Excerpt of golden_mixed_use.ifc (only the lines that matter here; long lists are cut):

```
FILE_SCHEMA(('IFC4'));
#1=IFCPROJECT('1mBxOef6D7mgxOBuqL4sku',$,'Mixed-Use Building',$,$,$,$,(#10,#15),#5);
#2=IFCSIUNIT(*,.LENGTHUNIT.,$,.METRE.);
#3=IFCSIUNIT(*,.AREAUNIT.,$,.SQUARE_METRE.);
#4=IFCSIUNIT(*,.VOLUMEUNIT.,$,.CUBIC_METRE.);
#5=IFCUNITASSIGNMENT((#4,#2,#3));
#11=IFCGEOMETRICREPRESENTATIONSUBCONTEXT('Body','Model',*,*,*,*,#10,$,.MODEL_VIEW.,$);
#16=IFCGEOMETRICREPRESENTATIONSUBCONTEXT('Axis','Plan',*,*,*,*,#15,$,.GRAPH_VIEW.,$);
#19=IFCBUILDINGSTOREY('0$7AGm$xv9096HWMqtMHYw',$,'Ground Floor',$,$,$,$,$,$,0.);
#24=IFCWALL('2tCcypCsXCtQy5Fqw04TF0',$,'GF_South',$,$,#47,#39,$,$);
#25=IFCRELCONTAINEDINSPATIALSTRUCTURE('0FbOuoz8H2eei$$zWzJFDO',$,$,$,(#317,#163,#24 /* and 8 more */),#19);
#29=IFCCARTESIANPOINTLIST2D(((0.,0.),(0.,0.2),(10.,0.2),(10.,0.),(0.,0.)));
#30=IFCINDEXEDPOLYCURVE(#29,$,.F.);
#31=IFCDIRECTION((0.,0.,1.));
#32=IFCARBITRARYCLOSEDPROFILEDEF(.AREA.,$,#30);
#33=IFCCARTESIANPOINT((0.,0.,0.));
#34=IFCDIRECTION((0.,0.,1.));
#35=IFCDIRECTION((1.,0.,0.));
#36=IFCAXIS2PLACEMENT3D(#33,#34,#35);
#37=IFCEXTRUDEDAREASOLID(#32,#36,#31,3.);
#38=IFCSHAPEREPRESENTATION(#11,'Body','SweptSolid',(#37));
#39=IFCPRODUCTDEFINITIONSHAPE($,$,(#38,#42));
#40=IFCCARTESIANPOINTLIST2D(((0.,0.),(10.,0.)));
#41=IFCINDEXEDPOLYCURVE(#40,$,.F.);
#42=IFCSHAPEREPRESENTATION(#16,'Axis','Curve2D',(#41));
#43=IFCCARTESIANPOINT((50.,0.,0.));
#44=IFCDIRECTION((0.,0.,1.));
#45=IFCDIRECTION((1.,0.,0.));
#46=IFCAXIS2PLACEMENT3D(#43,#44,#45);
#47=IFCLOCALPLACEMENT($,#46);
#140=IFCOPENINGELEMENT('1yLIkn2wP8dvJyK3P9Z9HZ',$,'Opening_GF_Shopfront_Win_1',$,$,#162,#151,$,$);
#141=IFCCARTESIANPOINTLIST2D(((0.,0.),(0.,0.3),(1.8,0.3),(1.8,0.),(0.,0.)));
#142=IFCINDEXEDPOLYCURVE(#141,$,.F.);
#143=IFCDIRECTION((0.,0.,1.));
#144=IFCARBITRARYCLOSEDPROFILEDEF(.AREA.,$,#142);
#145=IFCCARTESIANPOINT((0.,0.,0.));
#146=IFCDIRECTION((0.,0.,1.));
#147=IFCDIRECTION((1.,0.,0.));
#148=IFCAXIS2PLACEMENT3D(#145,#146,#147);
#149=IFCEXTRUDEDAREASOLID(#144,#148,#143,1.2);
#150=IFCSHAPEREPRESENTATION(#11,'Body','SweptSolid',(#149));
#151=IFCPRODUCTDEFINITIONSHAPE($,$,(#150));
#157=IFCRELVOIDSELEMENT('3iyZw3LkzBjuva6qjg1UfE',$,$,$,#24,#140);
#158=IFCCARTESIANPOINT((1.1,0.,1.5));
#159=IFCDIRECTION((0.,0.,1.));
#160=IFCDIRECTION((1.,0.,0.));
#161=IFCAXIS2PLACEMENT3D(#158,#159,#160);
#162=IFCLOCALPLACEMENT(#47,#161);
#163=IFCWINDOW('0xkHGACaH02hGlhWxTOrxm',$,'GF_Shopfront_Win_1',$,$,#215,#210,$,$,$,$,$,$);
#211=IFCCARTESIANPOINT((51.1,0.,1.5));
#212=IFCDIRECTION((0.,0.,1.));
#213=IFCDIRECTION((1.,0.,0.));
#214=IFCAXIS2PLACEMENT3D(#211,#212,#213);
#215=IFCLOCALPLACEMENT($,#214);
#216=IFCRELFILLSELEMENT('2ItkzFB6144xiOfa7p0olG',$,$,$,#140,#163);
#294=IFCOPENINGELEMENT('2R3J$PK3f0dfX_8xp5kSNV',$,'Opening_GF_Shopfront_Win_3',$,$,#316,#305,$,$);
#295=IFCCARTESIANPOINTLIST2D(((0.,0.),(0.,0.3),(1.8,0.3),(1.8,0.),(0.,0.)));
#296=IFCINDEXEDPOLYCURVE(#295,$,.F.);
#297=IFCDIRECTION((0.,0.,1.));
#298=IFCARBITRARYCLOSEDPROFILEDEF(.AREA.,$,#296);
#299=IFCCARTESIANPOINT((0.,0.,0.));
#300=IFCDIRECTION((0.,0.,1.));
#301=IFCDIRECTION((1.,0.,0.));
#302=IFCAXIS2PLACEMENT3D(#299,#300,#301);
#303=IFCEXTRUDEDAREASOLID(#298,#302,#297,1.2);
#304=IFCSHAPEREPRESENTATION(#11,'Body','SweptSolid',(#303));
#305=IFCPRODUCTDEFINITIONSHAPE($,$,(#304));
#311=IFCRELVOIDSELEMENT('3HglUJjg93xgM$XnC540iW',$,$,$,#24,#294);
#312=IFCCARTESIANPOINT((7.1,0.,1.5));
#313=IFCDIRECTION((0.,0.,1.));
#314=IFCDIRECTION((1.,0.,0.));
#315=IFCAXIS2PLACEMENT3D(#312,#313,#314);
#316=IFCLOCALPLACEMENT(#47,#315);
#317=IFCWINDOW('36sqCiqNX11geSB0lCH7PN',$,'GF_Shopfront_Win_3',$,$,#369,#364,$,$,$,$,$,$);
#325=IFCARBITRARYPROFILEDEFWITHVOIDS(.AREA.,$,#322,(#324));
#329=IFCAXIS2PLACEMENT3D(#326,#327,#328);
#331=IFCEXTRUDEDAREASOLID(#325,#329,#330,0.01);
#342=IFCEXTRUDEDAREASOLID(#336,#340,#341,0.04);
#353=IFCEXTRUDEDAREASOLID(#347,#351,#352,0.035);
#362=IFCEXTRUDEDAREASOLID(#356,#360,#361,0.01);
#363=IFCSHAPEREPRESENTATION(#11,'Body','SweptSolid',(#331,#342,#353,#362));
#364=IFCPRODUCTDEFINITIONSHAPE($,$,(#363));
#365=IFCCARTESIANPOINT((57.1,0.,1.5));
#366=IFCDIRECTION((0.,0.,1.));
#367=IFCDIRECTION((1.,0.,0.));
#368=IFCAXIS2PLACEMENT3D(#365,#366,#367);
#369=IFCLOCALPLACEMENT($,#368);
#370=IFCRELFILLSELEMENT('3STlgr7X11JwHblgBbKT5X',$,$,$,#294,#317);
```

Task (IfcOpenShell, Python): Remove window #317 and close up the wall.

```python
import ifcopenshell
import ifcopenshell.api.feature
import ifcopenshell.api.root
import ifcopenshell.geom
import ifcopenshell.util.shape

model = ifcopenshell.open("golden_mixed_use.ifc")
settings = ifcopenshell.geom.settings()


def volume(element):
    """Net volume in cubic metres, openings subtracted."""
    shape = ifcopenshell.geom.create_shape(settings, element)
    return ifcopenshell.util.shape.get_volume(shape.geometry)


window = model.by_guid("36sqCiqNX11geSB0lCH7PN")
opening = window.FillsVoids[0].RelatingOpeningElement
wall = opening.VoidsElements[0].RelatingBuildingElement
before = volume(wall)

ifcopenshell.api.root.remove_product(model, product=window)
ifcopenshell.api.feature.remove_feature(model, feature=opening)

after = volume(wall)

print(f"wall volume {before:.3f} -> {after:.3f} m3")

model.write("golden_mixed_use-out.ifc")
```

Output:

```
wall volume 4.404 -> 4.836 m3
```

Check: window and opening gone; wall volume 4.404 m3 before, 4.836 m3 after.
